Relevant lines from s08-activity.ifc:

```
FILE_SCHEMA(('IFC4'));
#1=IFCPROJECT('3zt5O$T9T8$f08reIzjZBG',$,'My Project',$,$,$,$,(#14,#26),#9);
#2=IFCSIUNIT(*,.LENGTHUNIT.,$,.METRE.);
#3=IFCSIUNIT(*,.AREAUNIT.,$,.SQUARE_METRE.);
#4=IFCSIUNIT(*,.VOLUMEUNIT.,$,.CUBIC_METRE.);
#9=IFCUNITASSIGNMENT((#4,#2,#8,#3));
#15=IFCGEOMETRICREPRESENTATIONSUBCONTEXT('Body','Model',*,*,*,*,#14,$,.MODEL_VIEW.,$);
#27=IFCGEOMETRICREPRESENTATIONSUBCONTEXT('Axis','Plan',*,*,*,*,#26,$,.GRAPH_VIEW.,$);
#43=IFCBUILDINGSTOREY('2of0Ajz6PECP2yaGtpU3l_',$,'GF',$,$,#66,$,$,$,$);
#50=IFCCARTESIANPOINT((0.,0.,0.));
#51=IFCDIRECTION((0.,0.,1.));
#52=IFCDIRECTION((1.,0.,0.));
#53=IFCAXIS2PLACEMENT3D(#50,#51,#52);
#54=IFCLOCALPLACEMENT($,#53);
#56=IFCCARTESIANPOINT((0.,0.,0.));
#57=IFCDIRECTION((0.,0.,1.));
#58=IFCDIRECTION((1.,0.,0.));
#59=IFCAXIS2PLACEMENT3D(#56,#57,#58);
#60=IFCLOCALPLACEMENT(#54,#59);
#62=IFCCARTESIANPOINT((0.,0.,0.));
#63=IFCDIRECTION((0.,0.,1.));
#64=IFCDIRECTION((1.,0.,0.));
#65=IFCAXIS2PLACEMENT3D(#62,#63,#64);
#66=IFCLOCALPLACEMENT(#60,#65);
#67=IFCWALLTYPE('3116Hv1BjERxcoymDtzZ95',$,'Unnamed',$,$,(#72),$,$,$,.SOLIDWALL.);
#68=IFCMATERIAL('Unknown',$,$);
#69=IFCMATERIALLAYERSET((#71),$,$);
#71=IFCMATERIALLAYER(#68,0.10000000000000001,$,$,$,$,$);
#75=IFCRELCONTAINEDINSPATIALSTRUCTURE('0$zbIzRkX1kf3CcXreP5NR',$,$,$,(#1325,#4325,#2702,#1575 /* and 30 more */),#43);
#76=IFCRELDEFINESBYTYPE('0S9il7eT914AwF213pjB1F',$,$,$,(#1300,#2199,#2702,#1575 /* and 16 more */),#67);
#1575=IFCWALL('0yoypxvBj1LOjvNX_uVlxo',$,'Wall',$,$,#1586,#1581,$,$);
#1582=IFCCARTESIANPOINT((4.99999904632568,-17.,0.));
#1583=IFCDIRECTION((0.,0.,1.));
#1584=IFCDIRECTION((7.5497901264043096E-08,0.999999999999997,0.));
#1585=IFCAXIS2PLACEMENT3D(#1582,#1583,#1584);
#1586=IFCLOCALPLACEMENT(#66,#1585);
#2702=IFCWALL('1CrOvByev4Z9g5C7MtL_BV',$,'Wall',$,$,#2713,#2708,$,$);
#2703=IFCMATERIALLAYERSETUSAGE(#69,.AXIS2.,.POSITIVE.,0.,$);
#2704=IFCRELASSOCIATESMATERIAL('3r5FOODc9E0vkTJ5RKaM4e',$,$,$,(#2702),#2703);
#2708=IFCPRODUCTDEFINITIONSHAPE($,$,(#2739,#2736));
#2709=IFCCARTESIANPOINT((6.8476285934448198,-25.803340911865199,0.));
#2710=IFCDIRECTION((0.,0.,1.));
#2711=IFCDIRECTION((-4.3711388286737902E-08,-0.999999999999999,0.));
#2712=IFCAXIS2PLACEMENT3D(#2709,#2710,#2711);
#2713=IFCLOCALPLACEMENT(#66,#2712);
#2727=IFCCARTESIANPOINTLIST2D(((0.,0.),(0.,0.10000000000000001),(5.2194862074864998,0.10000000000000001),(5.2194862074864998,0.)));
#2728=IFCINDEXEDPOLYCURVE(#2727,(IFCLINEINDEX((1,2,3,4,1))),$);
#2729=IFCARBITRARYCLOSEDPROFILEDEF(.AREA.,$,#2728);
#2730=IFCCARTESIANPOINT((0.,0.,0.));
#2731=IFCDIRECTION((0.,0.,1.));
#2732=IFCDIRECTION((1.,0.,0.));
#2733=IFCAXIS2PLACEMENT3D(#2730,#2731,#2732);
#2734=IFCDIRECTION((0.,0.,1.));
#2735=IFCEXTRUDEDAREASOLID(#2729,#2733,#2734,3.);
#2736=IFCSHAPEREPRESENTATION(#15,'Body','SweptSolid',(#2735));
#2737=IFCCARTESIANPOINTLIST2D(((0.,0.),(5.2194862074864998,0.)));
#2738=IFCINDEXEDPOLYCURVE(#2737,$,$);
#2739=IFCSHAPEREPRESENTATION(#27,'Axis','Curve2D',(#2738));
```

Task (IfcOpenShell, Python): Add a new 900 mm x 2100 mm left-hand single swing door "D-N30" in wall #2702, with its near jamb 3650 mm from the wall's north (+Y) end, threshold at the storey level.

```python
import numpy as np
import ifcopenshell
import ifcopenshell.api.feature
import ifcopenshell.api.geometry
import ifcopenshell.api.root
import ifcopenshell.api.spatial
import ifcopenshell.geom
import ifcopenshell.util.element
import ifcopenshell.util.placement
import ifcopenshell.util.representation
import ifcopenshell.util.shape
import ifcopenshell.util.unit

model = ifcopenshell.open("s08-activity.ifc")
unit_scale = ifcopenshell.util.unit.calculate_unit_scale(model)
settings = ifcopenshell.geom.settings()


def volume(element):
    """Net volume in cubic metres, openings subtracted."""
    shape = ifcopenshell.geom.create_shape(settings, element)
    return ifcopenshell.util.shape.get_volume(shape.geometry)


wall = model.by_guid("1CrOvByev4Z9g5C7MtL_BV")
storey = ifcopenshell.util.element.get_container(wall, ifc_class="IfcBuildingStorey")
context = ifcopenshell.util.representation.get_context(model, "Model", "Body", "MODEL_VIEW")
before = volume(wall)

width, height, from_end, sill = 0.9, 2.1, 3.65, 0.0  # metres

# The wall runs along its own X axis, and the end named is its -X end.
wall_shape = ifcopenshell.geom.create_shape(settings, wall)
x, y, z = ifcopenshell.util.shape.get_vertices(wall_shape.geometry).T
start = x.min() + from_end
face, thickness = float(y.min()), float(y.max() - y.min())
wall_matrix = ifcopenshell.util.placement.get_local_placement(wall.ObjectPlacement)
level = ifcopenshell.util.placement.get_local_placement(storey.ObjectPlacement)[2, 3]


def in_wall(x, y):
    """Placement at x, y metres in the wall's axes, at sill height."""
    matrix = wall_matrix.copy()
    matrix[:, 3] = wall_matrix @ np.array([x / unit_scale, y / unit_scale, 0.0, 1.0])
    matrix[2, 3] = level + sill / unit_scale
    return matrix


# Opening: a box that overshoots both wall faces by 50 mm.
opening = ifcopenshell.api.root.create_entity(model, ifc_class="IfcOpeningElement", predefined_type="OPENING")
box = ifcopenshell.api.geometry.add_wall_representation(
    model, context=context, length=width, height=height, thickness=thickness + 0.1
)
ifcopenshell.api.geometry.assign_representation(model, product=opening, representation=box)
ifcopenshell.api.geometry.edit_object_placement(model, product=opening, matrix=in_wall(start, face - 0.05), is_si=False)
ifcopenshell.api.feature.add_feature(model, feature=opening, element=wall)

door = ifcopenshell.api.root.create_entity(model, ifc_class="IfcDoor", name="D-N30", predefined_type="DOOR")
door.OverallWidth, door.OverallHeight = width / unit_scale, height / unit_scale
door.OperationType = "SINGLE_SWING_LEFT"
body = ifcopenshell.api.geometry.add_door_representation(
    model,
    context=context,
    overall_width=door.OverallWidth,
    overall_height=door.OverallHeight,
    operation_type="SINGLE_SWING_LEFT",
    lining_properties={"LiningDepth": thickness / unit_scale, "ThresholdDepth": thickness / unit_scale},
)
ifcopenshell.api.geometry.assign_representation(model, product=door, representation=body)
ifcopenshell.api.spatial.assign_container(model, products=[door], relating_structure=storey)
ifcopenshell.api.feature.add_filling(model, opening=opening, element=door)

# The lining spans the wall, so the door starts at the wall face.
ifcopenshell.api.geometry.edit_object_placement(model, product=door, matrix=in_wall(start, face), is_si=False)

after = volume(wall)

print(f"wall volume {before:.3f} -> {after:.3f} m3")

model.write("s08-activity_updated.ifc")
```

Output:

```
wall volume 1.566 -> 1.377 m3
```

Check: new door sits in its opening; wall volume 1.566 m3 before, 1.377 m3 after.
